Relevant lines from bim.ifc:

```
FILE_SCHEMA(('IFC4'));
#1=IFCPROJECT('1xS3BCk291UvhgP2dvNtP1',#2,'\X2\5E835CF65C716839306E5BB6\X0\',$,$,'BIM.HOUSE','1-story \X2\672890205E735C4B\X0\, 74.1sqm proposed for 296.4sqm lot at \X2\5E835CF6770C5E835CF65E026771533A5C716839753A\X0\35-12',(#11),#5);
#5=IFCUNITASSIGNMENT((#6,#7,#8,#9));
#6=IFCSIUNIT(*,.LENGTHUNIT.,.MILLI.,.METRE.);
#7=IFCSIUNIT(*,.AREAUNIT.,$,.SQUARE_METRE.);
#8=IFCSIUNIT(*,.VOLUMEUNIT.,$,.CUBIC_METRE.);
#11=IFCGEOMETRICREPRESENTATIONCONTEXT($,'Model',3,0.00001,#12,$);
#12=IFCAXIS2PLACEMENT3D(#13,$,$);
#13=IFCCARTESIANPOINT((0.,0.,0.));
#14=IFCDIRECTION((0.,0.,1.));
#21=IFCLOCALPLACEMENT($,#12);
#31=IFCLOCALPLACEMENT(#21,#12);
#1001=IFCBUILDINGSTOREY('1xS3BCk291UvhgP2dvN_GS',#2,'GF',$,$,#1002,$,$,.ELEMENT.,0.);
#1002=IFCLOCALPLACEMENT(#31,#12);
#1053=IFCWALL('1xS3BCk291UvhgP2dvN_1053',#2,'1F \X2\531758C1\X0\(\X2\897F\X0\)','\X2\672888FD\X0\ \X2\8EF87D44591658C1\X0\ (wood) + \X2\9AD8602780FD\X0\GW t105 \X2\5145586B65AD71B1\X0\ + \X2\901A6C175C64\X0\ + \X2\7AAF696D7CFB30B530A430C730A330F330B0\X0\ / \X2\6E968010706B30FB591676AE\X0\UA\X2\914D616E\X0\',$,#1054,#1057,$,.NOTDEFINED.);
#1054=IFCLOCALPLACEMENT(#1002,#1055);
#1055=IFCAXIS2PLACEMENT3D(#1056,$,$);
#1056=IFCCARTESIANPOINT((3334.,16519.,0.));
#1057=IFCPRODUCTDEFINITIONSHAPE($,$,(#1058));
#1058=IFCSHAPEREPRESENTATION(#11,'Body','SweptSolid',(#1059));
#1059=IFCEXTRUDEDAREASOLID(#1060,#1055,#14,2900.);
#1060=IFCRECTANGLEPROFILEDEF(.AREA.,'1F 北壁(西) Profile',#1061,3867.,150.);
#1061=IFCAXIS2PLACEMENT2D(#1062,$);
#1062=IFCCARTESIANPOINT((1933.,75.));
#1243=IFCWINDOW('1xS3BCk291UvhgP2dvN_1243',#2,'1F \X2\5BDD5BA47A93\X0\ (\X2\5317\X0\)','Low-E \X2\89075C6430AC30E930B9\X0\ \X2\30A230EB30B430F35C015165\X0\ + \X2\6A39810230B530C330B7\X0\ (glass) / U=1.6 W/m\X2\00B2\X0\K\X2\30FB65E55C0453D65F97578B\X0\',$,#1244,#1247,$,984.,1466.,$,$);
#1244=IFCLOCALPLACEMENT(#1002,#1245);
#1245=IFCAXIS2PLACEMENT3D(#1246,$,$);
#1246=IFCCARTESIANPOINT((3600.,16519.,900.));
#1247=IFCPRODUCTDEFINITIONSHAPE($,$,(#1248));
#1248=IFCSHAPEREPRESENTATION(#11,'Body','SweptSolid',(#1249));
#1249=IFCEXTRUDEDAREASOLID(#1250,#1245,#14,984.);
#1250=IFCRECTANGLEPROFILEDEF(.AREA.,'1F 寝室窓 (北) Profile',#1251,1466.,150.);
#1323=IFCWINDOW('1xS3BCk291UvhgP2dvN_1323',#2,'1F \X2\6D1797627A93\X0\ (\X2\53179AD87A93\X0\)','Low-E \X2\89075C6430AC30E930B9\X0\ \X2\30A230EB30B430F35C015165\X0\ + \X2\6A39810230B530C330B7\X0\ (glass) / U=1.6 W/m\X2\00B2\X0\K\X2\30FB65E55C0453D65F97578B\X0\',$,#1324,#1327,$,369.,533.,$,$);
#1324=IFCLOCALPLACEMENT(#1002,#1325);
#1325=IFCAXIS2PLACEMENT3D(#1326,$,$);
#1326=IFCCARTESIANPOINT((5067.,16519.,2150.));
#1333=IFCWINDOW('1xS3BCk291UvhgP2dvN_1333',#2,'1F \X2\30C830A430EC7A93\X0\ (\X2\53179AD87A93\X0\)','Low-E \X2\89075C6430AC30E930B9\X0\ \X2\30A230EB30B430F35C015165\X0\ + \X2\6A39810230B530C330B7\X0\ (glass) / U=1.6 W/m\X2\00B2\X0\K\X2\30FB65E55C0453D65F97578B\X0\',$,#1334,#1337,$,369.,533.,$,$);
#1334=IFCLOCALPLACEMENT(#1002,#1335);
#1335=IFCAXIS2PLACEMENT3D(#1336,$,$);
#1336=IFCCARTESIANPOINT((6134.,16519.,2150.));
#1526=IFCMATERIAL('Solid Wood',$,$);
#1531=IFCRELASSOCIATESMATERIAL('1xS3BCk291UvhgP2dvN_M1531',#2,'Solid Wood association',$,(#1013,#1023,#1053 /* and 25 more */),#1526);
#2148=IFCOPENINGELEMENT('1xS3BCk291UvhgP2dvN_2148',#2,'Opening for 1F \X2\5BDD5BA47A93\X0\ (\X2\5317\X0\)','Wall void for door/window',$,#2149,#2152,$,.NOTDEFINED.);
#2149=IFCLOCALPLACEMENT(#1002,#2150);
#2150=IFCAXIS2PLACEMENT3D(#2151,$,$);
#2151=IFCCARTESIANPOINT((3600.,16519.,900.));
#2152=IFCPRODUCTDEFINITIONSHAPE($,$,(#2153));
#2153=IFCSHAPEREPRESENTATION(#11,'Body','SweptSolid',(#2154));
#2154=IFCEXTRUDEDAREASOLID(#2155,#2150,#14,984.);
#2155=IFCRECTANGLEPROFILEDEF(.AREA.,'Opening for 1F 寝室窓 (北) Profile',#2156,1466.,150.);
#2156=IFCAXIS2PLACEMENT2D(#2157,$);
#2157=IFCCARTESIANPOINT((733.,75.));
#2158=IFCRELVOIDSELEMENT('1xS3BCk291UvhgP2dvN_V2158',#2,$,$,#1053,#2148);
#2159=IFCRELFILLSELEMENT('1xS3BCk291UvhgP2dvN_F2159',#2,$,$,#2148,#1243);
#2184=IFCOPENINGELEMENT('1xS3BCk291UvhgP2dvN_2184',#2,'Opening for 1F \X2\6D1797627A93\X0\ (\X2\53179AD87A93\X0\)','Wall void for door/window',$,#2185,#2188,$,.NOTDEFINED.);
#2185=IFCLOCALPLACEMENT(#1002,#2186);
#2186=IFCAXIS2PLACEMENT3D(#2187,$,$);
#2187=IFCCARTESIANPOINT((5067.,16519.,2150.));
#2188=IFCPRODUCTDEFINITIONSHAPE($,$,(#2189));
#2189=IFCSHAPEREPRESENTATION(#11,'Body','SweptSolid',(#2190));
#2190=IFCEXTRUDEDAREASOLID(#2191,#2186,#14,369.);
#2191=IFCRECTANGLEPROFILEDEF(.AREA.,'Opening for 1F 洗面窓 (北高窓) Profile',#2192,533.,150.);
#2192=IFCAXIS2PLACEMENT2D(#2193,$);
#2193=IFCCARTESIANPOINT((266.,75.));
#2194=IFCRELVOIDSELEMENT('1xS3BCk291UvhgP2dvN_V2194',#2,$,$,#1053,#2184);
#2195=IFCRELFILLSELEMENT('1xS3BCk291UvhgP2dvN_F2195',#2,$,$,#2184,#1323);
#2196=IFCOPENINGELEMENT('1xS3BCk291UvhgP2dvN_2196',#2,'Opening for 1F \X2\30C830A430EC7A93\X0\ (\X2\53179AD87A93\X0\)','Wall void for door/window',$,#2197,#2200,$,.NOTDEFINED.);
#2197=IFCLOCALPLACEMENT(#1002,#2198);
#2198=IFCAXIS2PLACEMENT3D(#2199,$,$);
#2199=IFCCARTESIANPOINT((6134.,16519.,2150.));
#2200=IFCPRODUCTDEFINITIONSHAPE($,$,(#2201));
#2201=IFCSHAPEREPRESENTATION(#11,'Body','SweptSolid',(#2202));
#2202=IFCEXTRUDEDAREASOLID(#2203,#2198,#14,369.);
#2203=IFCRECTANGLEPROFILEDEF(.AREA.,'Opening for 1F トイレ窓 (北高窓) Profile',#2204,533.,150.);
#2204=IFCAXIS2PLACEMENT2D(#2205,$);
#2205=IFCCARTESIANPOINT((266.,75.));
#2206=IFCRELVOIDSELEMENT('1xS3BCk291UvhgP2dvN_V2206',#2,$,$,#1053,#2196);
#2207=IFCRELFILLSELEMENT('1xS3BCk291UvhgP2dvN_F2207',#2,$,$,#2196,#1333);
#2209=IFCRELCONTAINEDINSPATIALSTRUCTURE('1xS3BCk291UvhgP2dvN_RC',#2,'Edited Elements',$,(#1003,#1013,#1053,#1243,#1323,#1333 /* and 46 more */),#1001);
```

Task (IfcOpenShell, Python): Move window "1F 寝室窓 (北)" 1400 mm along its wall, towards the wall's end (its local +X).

```python
import ifcopenshell
import ifcopenshell.api.geometry
import ifcopenshell.util.placement

model = ifcopenshell.open("bim.ifc")

window = model.by_guid("1xS3BCk291UvhgP2dvN_1243")
opening = window.FillsVoids[0].RelatingOpeningElement
wall = opening.VoidsElements[0].RelatingBuildingElement

wall_matrix = ifcopenshell.util.placement.get_local_placement(wall.ObjectPlacement)
shift = wall_matrix[:3, 0] * 1400.0
before = ifcopenshell.util.placement.get_local_placement(window.ObjectPlacement)[:3, 3].copy()

# The window is not placed relative to its opening, so move both.
for product in (opening, window):
    matrix = ifcopenshell.util.placement.get_local_placement(product.ObjectPlacement)
    matrix[:3, 3] += shift
    ifcopenshell.api.geometry.edit_object_placement(model, product=product, matrix=matrix, is_si=False)

after = ifcopenshell.util.placement.get_local_placement(window.ObjectPlacement)[:3, 3]
print("window moved by", (after - before).round(3) + 0.0)

model.write("bim_v2.ifc")
```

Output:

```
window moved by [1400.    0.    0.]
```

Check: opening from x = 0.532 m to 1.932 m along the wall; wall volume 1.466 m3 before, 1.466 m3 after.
